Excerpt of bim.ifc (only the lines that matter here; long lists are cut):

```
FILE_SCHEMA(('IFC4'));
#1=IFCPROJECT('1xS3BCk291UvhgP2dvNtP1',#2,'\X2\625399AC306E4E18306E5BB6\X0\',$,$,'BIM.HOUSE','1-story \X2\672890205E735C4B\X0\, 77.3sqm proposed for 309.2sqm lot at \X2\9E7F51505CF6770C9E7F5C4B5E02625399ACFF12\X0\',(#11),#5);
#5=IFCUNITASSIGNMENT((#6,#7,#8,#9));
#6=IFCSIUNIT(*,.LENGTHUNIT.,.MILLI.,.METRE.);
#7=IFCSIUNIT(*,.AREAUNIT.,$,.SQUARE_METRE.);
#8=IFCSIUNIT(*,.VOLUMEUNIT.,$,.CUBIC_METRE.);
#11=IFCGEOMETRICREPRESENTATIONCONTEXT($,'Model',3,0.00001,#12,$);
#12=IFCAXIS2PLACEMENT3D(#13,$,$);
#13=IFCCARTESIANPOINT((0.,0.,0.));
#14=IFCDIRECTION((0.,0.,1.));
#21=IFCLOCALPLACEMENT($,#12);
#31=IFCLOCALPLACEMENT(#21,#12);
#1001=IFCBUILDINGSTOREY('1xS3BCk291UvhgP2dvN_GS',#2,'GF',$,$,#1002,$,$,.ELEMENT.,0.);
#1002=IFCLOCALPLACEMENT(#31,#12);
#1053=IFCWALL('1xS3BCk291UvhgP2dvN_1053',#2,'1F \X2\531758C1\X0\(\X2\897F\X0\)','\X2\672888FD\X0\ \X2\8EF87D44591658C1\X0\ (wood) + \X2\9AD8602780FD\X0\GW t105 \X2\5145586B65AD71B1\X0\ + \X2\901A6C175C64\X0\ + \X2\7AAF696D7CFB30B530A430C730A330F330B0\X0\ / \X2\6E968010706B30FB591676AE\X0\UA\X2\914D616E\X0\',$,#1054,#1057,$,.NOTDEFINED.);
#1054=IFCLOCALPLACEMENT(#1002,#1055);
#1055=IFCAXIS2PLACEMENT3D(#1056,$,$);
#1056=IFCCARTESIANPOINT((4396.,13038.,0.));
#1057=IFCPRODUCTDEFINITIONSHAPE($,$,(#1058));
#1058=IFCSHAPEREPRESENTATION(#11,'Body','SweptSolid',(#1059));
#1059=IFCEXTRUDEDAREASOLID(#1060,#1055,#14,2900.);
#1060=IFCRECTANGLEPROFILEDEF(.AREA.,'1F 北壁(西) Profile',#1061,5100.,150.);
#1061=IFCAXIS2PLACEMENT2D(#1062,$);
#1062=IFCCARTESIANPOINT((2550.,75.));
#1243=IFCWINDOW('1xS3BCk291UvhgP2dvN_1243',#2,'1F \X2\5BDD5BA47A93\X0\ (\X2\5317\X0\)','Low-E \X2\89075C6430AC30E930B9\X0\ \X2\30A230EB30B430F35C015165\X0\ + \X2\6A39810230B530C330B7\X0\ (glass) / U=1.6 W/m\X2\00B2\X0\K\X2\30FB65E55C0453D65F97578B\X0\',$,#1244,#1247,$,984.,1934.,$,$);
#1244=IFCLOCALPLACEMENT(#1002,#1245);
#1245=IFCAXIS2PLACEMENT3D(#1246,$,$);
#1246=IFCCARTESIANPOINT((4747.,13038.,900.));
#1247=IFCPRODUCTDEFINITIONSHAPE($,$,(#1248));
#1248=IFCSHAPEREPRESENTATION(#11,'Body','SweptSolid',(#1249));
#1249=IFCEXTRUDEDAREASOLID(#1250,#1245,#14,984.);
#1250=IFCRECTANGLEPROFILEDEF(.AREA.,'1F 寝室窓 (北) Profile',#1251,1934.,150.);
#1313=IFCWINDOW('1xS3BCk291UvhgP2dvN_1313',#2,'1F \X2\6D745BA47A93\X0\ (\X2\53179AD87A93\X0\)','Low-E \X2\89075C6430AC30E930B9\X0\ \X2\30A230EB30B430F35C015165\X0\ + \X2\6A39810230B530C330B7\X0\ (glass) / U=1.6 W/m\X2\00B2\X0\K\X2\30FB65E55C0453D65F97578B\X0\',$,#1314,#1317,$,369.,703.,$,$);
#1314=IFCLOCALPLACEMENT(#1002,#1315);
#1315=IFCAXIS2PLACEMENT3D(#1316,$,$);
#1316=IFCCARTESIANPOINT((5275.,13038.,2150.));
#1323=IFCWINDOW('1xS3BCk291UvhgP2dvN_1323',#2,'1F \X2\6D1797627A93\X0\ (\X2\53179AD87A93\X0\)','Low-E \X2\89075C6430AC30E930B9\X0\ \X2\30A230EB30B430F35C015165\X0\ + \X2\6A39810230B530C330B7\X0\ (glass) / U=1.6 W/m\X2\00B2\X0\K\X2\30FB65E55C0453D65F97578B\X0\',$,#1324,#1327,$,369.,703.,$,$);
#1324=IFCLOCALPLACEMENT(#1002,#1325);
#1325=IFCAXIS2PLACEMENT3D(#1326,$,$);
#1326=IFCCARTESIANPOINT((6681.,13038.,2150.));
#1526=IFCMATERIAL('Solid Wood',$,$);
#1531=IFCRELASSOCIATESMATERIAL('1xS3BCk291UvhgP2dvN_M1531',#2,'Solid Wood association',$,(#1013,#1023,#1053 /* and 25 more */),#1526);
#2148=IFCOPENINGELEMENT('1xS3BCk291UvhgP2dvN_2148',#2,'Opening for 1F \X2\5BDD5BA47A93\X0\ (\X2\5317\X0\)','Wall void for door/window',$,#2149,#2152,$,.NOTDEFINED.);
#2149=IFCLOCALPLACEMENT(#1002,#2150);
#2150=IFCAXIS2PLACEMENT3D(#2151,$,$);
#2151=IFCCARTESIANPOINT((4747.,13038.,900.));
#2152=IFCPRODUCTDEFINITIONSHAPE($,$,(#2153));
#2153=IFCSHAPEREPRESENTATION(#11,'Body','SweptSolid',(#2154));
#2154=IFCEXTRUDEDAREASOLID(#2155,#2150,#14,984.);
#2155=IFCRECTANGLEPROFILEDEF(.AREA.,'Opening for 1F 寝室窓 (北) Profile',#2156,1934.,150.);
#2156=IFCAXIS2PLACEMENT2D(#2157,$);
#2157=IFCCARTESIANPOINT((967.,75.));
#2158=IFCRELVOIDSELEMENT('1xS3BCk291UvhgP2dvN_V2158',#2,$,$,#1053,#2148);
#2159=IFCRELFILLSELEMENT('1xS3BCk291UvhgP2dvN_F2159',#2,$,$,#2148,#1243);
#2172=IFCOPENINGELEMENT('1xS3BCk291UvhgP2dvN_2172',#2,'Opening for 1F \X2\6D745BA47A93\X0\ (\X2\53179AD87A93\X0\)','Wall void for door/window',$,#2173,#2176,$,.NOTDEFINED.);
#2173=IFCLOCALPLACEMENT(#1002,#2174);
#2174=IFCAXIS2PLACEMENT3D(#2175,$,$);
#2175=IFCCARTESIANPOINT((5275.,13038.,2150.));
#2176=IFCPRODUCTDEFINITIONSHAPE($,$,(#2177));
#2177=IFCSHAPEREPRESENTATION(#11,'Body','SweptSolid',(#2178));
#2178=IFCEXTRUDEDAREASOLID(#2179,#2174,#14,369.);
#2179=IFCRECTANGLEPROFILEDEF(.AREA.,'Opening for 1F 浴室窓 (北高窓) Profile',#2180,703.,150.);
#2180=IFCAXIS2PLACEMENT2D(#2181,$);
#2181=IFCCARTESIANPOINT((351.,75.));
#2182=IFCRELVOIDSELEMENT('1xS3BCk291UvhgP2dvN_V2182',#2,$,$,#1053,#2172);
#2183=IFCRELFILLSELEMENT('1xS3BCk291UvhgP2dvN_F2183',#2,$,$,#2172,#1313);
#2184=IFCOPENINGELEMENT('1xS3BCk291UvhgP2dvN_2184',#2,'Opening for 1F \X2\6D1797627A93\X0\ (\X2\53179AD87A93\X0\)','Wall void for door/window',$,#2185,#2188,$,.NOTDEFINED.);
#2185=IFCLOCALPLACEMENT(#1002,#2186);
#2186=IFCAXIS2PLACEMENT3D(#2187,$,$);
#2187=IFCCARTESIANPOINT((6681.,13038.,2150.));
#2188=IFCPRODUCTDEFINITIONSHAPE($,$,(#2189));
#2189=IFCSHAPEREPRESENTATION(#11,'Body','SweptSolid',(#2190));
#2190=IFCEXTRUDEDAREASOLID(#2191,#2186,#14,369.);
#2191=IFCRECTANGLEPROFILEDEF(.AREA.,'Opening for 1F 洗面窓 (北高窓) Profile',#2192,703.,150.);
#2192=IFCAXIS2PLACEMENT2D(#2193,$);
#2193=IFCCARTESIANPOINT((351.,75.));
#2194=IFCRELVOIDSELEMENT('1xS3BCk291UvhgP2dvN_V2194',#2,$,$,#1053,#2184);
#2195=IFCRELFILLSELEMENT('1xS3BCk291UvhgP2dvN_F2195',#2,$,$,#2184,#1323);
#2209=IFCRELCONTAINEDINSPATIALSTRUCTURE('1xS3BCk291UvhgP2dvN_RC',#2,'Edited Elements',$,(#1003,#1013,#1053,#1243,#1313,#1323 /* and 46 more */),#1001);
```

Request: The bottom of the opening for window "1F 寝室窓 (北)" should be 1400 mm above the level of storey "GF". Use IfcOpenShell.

```python
import numpy as np
import ifcopenshell
import ifcopenshell.api.geometry
import ifcopenshell.geom
import ifcopenshell.util.element
import ifcopenshell.util.placement
import ifcopenshell.util.shape
import ifcopenshell.util.unit

model = ifcopenshell.open("bim.ifc")
unit_scale = ifcopenshell.util.unit.calculate_unit_scale(model)

window = model.by_id(1243)
opening = window.FillsVoids[0].RelatingOpeningElement
storey = ifcopenshell.util.element.get_container(window, ifc_class="IfcBuildingStorey")
level = ifcopenshell.util.placement.get_local_placement(storey.ObjectPlacement)[2, 3]

# The opening's origin need not be at the sill, so measure its lowest point.
shape = ifcopenshell.geom.create_shape(ifcopenshell.geom.settings(), opening)
bottom = ifcopenshell.util.shape.get_shape_bottom_elevation(shape, shape.geometry) / unit_scale
dz = level + 1.4 / unit_scale - bottom

shift = np.array([0.0, 0.0, dz])
# The window is not placed relative to its opening, so move both.
for product in (opening, window):
    matrix = ifcopenshell.util.placement.get_local_placement(product.ObjectPlacement)
    matrix[:3, 3] += shift
    ifcopenshell.api.geometry.edit_object_placement(model, product=product, matrix=matrix, is_si=False)

print(f"moved by {dz * unit_scale:+.3f} m")

model.write("bim_rev.ifc")
```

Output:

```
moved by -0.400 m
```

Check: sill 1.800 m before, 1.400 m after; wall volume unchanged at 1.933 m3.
